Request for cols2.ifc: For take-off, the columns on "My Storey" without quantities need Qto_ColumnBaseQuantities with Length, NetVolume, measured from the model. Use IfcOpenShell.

First a look at what the model holds.

```python
import ifcopenshell
import ifcopenshell.util.element
import ifcopenshell.util.unit

model = ifcopenshell.open("cols2.ifc")
print(model.schema)
for unit_type in ("LENGTHUNIT", "AREAUNIT", "VOLUMEUNIT"):
    print(unit_type, ifcopenshell.util.unit.calculate_unit_scale(model, unit_type))
storey = next(s for s in model.by_type("IfcBuildingStorey") if s.Name == "My Storey")
columns = [e for e in ifcopenshell.util.element.get_decomposition(storey) if e.is_a("IfcColumn")]
for e in sorted(columns, key=lambda e: e.id()):
    print(e.id(), e.is_a(), e.Name, list(ifcopenshell.util.element.get_psets(e, qtos_only=True)), sep=" | ")
```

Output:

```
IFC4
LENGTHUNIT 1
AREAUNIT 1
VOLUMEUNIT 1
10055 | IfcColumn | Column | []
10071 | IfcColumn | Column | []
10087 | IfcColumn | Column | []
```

```python
import ifcopenshell
import ifcopenshell.api.pset
import ifcopenshell.geom
import ifcopenshell.util.element
import ifcopenshell.util.shape
import ifcopenshell.util.unit

model = ifcopenshell.open("cols2.ifc")
unit_scale = ifcopenshell.util.unit.calculate_unit_scale(model)
volume_scale = ifcopenshell.util.unit.calculate_unit_scale(model, "VOLUMEUNIT")
settings = ifcopenshell.geom.settings()

storey = next(s for s in model.by_type("IfcBuildingStorey") if s.Name == "My Storey")
columns = [e for e in ifcopenshell.util.element.get_decomposition(storey) if e.is_a("IfcColumn")]

for e in sorted(columns, key=lambda e: e.id()):
    if ifcopenshell.util.element.get_psets(e, qtos_only=True, should_inherit=False):
        continue
    # Geometry comes back in metres, in the element's own axes.
    shape = ifcopenshell.geom.create_shape(settings, e)
    values = {
        "Length": ifcopenshell.util.shape.get_z(shape.geometry) / unit_scale,
        "NetVolume": ifcopenshell.util.shape.get_volume(shape.geometry) / volume_scale,
    }
    qto = ifcopenshell.api.pset.add_qto(model, product=e, name="Qto_ColumnBaseQuantities")
    ifcopenshell.api.pset.edit_qto(model, qto=qto, properties=values)
    print(e.id(), {k: round(v, 3) for k, v in values.items()})

model.write("cols2-out.ifc")
```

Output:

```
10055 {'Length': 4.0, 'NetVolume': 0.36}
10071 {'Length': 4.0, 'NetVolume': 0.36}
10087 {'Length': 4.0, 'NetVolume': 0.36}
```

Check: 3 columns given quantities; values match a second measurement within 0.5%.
